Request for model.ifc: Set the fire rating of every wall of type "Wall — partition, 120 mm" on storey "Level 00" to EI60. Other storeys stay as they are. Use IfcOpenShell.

First a look at what the model holds.

```python
import ifcopenshell
import ifcopenshell.util.element

model = ifcopenshell.open("model.ifc")
print(model.schema)
storey = next(s for s in model.by_type("IfcBuildingStorey") if s.Name == "Level 00")
walls = [e for e in ifcopenshell.util.element.get_decomposition(storey) if e.is_a("IfcWall")]
seen = {}
for e in walls:
    element_type = ifcopenshell.util.element.get_type(e)
    key = (element_type.Name if element_type != e and element_type else None, ifcopenshell.util.element.get_pset(e, "Pset_WallCommon", "FireRating"))
    seen[key] = seen.get(key, 0) + 1
for (name, value), count in sorted(seen.items(), key=str):
    print(count, "x", name, "|", value)
```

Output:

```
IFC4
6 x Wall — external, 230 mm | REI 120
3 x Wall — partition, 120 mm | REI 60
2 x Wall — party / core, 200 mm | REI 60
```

```python
import ifcopenshell
import ifcopenshell.api.pset
import ifcopenshell.util.element

model = ifcopenshell.open("model.ifc")

storey = next(s for s in model.by_type("IfcBuildingStorey") if s.Name == "Level 00")
walls = [e for e in ifcopenshell.util.element.get_decomposition(storey) if e.is_a("IfcWall")]

count = 0
for e in walls:
    element_type = ifcopenshell.util.element.get_type(e)
    if element_type in (None, e) or element_type.Name != "Wall — partition, 120 mm":
        continue
    # add_pset returns the element's existing set when there is one.
    pset = ifcopenshell.api.pset.add_pset(model, product=e, name="Pset_WallCommon")
    ifcopenshell.api.pset.edit_pset(model, pset=pset, properties={"FireRating": "EI60"})
    count += 1

print(count, "walls updated")

model.write("model_v2.ifc")
```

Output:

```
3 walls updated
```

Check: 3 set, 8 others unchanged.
